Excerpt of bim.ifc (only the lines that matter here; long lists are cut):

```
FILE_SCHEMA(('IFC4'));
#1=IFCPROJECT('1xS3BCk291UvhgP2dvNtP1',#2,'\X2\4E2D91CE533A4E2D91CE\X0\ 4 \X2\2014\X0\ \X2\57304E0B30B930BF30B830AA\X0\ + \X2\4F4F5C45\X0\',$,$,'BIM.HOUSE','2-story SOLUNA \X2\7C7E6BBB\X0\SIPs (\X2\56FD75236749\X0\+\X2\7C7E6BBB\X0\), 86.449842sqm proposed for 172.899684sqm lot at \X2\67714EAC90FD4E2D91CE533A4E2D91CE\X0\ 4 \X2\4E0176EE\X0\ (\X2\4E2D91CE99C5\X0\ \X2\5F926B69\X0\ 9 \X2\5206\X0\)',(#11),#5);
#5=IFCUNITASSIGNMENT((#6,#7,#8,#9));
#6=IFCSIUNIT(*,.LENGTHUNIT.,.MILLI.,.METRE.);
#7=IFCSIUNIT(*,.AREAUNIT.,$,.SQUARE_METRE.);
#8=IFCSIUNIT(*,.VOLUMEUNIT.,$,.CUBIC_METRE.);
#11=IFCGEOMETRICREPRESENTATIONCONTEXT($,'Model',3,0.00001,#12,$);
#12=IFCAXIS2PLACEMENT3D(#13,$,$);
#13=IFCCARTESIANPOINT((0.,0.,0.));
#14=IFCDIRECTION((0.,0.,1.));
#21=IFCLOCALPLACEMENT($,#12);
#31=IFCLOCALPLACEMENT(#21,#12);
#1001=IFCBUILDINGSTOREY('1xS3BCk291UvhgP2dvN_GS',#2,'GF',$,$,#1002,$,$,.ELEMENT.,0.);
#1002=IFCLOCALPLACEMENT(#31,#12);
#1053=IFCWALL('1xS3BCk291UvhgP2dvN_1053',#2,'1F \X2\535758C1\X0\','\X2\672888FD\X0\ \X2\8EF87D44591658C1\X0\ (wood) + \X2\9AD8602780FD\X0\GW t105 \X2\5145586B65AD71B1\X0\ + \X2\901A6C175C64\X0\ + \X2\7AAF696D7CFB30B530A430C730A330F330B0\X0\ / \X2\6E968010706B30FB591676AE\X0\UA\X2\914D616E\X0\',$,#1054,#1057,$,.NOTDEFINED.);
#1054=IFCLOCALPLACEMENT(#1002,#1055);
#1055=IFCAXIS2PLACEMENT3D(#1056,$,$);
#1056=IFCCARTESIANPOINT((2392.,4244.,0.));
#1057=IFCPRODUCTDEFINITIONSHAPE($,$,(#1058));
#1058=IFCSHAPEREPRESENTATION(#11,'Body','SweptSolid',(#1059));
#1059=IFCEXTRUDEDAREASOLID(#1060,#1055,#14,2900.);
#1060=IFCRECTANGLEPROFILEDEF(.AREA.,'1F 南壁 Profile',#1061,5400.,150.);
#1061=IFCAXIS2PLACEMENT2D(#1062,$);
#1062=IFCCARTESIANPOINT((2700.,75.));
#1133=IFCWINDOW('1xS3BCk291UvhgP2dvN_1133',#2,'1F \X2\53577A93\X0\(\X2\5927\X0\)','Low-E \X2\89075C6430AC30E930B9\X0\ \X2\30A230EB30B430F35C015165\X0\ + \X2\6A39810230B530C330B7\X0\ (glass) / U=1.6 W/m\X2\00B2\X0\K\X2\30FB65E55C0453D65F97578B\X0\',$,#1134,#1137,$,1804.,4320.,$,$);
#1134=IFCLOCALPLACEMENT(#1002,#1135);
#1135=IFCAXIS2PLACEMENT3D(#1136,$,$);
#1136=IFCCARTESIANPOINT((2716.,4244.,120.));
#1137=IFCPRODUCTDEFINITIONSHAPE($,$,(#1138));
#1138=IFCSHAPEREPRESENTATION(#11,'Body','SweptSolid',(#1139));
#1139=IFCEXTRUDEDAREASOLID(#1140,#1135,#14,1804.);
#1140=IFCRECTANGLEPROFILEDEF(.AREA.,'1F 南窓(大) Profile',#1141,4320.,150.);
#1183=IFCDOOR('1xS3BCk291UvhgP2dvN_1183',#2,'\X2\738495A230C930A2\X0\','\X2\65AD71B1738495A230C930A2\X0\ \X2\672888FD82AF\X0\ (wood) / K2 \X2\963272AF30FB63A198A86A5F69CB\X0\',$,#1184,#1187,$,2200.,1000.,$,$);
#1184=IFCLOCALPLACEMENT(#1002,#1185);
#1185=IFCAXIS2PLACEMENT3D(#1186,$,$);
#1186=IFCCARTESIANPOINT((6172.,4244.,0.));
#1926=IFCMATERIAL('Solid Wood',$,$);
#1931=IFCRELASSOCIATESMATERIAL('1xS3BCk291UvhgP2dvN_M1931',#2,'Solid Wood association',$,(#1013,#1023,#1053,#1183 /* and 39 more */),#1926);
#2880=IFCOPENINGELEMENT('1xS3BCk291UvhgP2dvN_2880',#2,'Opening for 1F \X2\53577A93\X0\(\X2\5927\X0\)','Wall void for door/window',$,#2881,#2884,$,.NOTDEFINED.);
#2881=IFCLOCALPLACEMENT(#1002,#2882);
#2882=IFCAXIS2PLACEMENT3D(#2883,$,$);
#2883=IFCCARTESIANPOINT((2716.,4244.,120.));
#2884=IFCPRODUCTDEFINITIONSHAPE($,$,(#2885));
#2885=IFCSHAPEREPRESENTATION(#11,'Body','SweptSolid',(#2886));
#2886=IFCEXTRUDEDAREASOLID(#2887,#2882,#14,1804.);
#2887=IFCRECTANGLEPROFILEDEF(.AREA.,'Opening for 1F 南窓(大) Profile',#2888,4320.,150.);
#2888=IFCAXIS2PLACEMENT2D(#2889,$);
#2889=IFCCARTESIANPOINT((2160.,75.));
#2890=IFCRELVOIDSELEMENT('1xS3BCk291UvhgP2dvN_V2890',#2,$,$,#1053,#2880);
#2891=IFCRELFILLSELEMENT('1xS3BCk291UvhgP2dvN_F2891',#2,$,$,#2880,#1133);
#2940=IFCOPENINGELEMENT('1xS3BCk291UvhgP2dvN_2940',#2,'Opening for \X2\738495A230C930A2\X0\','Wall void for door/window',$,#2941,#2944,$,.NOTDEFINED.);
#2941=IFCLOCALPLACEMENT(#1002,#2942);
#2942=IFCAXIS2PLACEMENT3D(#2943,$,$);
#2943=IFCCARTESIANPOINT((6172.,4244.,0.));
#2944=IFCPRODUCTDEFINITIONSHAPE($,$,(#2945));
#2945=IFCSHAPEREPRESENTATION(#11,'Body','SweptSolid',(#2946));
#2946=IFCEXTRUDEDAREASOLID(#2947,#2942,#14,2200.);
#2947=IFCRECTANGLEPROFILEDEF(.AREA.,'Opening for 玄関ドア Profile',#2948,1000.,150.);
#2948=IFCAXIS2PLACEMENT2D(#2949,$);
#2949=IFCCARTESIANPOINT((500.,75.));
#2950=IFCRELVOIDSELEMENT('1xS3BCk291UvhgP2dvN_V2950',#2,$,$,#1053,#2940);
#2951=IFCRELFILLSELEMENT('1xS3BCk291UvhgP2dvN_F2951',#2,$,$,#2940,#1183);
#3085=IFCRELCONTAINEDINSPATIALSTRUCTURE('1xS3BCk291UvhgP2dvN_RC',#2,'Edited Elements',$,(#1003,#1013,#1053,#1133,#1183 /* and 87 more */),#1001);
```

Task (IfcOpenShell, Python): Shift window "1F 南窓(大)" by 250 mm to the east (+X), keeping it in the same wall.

```python
import ifcopenshell
import ifcopenshell.api.geometry
import ifcopenshell.util.placement

model = ifcopenshell.open("bim.ifc")

window = model.by_id(1133)
opening = window.FillsVoids[0].RelatingOpeningElement
wall = opening.VoidsElements[0].RelatingBuildingElement

wall_matrix = ifcopenshell.util.placement.get_local_placement(wall.ObjectPlacement)
shift = wall_matrix[:3, 0] * 250.0
before = ifcopenshell.util.placement.get_local_placement(window.ObjectPlacement)[:3, 3].copy()

# The window is not placed relative to its opening, so move both.
for product in (opening, window):
    matrix = ifcopenshell.util.placement.get_local_placement(product.ObjectPlacement)
    matrix[:3, 3] += shift
    ifcopenshell.api.geometry.edit_object_placement(model, product=product, matrix=matrix, is_si=False)

after = ifcopenshell.util.placement.get_local_placement(window.ObjectPlacement)[:3, 3]
print("window moved by", (after - before).round(3) + 0.0)

model.write("bim_v2.ifc")
```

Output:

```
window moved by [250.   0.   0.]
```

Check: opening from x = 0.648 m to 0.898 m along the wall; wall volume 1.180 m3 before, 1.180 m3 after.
